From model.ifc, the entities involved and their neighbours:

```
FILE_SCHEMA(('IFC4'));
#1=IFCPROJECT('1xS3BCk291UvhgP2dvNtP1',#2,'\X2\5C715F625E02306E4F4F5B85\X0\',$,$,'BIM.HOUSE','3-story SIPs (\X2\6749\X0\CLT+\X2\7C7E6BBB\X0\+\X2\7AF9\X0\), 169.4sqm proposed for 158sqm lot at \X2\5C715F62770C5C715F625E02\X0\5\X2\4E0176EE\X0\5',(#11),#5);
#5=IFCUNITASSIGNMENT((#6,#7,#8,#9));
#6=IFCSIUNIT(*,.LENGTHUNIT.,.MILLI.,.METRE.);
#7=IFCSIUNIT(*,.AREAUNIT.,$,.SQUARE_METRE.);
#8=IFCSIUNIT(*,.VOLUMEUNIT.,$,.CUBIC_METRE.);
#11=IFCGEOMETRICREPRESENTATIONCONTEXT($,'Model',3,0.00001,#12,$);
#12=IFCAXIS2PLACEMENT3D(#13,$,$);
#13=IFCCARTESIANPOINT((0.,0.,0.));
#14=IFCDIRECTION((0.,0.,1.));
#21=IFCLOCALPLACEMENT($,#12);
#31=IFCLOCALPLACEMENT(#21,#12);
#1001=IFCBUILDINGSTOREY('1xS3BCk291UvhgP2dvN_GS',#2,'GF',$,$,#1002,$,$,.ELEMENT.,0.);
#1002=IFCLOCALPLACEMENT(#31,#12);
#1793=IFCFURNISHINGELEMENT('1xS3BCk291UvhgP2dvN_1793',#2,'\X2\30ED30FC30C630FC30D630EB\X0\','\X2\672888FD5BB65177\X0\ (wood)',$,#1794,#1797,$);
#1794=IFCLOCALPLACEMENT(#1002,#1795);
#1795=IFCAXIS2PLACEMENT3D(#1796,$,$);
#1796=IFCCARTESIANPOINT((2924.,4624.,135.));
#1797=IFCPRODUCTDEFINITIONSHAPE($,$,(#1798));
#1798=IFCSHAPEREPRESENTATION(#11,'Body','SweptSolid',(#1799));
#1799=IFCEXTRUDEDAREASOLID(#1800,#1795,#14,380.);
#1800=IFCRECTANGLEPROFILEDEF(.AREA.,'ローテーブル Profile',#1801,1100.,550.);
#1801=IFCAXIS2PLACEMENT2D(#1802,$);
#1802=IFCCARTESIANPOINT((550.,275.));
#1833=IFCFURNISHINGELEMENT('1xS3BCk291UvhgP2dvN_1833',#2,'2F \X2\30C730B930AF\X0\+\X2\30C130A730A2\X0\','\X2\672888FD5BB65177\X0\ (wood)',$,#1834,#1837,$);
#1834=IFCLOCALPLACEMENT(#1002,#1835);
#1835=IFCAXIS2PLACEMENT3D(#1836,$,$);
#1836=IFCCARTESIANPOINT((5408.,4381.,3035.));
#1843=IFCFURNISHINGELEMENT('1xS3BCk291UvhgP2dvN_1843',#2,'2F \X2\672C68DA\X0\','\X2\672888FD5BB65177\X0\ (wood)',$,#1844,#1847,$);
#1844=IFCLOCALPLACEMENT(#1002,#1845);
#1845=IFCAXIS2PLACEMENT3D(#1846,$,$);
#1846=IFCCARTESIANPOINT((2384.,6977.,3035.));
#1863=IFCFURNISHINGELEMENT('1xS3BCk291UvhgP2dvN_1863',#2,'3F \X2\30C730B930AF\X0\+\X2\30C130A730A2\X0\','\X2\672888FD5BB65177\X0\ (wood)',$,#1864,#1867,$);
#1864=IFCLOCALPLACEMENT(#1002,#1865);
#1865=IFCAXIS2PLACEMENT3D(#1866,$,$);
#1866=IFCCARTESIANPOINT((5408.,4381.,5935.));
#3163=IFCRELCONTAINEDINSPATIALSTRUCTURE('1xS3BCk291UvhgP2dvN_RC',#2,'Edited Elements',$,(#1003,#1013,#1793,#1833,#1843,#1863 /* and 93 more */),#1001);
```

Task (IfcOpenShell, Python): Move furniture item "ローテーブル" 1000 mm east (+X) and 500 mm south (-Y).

```python
import ifcopenshell
import ifcopenshell.api.geometry
import ifcopenshell.util.placement

model = ifcopenshell.open("model.ifc")

item = model.by_guid("1xS3BCk291UvhgP2dvN_1793")
matrix = ifcopenshell.util.placement.get_local_placement(item.ObjectPlacement)
matrix[0, 3] += 1000.0
matrix[1, 3] -= 500.0
ifcopenshell.api.geometry.edit_object_placement(model, product=item, matrix=matrix, is_si=False)

print(ifcopenshell.util.placement.get_local_placement(item.ObjectPlacement).round(3) + 0.0)

model.write("model_updated.ifc")
```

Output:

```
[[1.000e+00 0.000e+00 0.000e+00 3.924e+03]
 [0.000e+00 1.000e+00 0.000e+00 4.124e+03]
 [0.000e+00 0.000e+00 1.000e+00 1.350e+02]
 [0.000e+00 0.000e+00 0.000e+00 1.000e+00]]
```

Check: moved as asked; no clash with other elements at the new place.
